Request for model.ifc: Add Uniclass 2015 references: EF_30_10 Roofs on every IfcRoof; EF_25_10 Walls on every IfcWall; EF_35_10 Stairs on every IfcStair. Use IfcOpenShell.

First a look at what the model holds.

```python
import ifcopenshell

model = ifcopenshell.open("model.ifc")
print(model.schema)
print("classifications:", [c.Name for c in model.by_type("IfcClassification")])
for ifc_class in ("IfcDoor", "IfcRoof", "IfcStair", "IfcWall", "IfcWindow"):
    print(ifc_class, len(model.by_type(ifc_class)))
```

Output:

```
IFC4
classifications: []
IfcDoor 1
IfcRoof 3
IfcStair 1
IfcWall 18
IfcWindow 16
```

```python
import ifcopenshell
import ifcopenshell.api.classification

model = ifcopenshell.open("model.ifc")

system = ifcopenshell.api.classification.add_classification(model, classification="Uniclass 2015")

codes = {
    "IfcRoof": ("EF_30_10", "Roofs"),
    "IfcWall": ("EF_25_10", "Walls"),
    "IfcStair": ("EF_35_10", "Stairs"),
}
for ifc_class, (code, name) in codes.items():
    products = model.by_type(ifc_class)
    ifcopenshell.api.classification.add_reference(
        model, products=products, classification=system, identification=code, name=name
    )
    print(code, len(products))

model.write("model-out.ifc")
```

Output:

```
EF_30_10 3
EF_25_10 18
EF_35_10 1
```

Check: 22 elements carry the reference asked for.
